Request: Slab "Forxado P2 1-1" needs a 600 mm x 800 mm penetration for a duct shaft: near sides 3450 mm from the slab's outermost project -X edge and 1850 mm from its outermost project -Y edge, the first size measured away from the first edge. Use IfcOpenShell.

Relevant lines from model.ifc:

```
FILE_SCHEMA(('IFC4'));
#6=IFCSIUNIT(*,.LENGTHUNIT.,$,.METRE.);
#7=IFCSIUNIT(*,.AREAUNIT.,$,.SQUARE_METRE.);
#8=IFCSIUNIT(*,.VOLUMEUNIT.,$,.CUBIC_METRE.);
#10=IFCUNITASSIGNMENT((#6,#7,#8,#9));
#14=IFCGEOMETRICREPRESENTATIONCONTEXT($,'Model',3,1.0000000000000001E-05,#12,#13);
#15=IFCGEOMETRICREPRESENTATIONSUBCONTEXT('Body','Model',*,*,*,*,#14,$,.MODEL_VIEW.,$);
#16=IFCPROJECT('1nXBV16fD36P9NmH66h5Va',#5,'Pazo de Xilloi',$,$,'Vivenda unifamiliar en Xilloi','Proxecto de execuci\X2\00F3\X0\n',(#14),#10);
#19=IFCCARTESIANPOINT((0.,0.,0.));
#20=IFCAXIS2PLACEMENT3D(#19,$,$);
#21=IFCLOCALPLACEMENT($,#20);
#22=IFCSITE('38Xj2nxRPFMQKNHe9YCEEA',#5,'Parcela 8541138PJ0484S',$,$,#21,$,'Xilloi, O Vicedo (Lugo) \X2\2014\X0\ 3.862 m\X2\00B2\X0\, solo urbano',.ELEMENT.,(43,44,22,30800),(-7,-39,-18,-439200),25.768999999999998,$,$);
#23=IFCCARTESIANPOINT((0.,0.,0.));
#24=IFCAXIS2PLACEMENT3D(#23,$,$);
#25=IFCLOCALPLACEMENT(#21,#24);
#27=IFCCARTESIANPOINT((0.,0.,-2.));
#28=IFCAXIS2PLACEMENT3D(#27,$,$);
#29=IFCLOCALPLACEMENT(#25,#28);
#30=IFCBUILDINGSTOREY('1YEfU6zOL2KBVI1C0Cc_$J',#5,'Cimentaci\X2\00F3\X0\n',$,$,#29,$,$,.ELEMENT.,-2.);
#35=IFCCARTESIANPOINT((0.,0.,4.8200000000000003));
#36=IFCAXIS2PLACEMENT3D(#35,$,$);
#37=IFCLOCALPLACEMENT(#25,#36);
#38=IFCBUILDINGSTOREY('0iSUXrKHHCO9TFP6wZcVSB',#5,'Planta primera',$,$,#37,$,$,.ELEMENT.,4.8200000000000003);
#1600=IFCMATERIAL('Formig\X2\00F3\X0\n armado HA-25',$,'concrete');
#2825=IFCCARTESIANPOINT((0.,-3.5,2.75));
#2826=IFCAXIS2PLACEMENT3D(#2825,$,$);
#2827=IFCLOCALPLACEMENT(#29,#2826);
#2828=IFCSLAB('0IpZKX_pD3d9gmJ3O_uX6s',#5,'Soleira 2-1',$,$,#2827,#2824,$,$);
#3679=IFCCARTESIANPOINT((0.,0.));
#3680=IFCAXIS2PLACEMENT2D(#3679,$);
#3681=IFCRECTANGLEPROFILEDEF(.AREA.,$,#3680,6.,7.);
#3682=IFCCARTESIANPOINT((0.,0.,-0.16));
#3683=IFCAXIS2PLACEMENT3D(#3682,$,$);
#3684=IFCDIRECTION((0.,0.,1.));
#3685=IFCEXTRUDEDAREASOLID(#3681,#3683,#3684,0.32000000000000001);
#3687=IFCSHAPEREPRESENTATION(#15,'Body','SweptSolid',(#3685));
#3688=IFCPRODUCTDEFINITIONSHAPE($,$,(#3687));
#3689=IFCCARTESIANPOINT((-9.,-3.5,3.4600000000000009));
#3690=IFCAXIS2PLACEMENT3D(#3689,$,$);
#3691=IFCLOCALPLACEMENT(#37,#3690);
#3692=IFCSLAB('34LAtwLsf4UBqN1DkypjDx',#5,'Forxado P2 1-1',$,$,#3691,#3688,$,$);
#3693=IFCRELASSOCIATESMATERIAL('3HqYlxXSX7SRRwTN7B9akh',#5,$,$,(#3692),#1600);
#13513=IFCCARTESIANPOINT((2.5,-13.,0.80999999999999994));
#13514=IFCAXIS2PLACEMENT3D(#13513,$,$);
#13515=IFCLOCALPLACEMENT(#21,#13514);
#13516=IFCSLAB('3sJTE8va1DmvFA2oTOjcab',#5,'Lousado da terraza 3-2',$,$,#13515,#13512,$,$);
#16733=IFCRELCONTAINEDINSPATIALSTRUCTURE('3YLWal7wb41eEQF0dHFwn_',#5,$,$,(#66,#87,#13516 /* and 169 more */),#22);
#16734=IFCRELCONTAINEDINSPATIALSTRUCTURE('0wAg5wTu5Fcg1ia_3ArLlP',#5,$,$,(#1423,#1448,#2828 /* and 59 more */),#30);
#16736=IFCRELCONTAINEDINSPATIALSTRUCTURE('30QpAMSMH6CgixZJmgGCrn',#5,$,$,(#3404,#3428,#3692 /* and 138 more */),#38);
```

```python
import numpy as np
import ifcopenshell
import ifcopenshell.api.feature
import ifcopenshell.api.geometry
import ifcopenshell.api.root
import ifcopenshell.geom
import ifcopenshell.util.placement
import ifcopenshell.util.representation
import ifcopenshell.util.shape
import ifcopenshell.util.unit

model = ifcopenshell.open("model.ifc")
unit_scale = ifcopenshell.util.unit.calculate_unit_scale(model)
settings = ifcopenshell.geom.settings()


def volume(element):
    """Net volume in cubic metres, openings subtracted."""
    shape = ifcopenshell.geom.create_shape(settings, element)
    return ifcopenshell.util.shape.get_volume(shape.geometry)


slab = model.by_id(3692)
before = volume(slab)

# Extent in the slab's own axes, in metres. The edges named are its -X and -Y sides.
slab_shape = ifcopenshell.geom.create_shape(settings, slab)
vertices = ifcopenshell.util.shape.get_vertices(slab_shape.geometry)
x_min, y_min, bottom = vertices.min(axis=0)
top = vertices[:, 2].max()

opening = ifcopenshell.api.root.create_entity(model, ifc_class="IfcOpeningElement", name="Duct shaft opening", predefined_type="OPENING")
context = ifcopenshell.util.representation.get_context(model, "Model", "Body", "MODEL_VIEW")
width, depth = 0.6, 0.8
outline = [(0.0, 0.0), (width, 0.0), (width, depth), (0.0, depth), (0.0, 0.0)]
# Overshoot both faces by 50 mm so the cut is clean.
shape = ifcopenshell.api.geometry.add_slab_representation(
    model, context=context, depth=top - bottom + 0.1, polyline=outline
)
ifcopenshell.api.geometry.assign_representation(model, product=opening, representation=shape)

matrix = ifcopenshell.util.placement.get_local_placement(slab.ObjectPlacement)
matrix[:, 3] = matrix @ np.append(np.array([x_min + 3.45, y_min + 1.85, bottom - 0.05]) / unit_scale, 1.0)
ifcopenshell.api.geometry.edit_object_placement(model, product=opening, matrix=matrix, is_si=False)
ifcopenshell.api.feature.add_feature(model, feature=opening, element=slab)

after = volume(slab)

print(f"slab volume {before:.3f} -> {after:.3f} m3")

model.write("model_v2.ifc")
```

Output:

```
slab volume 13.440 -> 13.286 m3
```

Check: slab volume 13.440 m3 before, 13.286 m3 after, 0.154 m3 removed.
